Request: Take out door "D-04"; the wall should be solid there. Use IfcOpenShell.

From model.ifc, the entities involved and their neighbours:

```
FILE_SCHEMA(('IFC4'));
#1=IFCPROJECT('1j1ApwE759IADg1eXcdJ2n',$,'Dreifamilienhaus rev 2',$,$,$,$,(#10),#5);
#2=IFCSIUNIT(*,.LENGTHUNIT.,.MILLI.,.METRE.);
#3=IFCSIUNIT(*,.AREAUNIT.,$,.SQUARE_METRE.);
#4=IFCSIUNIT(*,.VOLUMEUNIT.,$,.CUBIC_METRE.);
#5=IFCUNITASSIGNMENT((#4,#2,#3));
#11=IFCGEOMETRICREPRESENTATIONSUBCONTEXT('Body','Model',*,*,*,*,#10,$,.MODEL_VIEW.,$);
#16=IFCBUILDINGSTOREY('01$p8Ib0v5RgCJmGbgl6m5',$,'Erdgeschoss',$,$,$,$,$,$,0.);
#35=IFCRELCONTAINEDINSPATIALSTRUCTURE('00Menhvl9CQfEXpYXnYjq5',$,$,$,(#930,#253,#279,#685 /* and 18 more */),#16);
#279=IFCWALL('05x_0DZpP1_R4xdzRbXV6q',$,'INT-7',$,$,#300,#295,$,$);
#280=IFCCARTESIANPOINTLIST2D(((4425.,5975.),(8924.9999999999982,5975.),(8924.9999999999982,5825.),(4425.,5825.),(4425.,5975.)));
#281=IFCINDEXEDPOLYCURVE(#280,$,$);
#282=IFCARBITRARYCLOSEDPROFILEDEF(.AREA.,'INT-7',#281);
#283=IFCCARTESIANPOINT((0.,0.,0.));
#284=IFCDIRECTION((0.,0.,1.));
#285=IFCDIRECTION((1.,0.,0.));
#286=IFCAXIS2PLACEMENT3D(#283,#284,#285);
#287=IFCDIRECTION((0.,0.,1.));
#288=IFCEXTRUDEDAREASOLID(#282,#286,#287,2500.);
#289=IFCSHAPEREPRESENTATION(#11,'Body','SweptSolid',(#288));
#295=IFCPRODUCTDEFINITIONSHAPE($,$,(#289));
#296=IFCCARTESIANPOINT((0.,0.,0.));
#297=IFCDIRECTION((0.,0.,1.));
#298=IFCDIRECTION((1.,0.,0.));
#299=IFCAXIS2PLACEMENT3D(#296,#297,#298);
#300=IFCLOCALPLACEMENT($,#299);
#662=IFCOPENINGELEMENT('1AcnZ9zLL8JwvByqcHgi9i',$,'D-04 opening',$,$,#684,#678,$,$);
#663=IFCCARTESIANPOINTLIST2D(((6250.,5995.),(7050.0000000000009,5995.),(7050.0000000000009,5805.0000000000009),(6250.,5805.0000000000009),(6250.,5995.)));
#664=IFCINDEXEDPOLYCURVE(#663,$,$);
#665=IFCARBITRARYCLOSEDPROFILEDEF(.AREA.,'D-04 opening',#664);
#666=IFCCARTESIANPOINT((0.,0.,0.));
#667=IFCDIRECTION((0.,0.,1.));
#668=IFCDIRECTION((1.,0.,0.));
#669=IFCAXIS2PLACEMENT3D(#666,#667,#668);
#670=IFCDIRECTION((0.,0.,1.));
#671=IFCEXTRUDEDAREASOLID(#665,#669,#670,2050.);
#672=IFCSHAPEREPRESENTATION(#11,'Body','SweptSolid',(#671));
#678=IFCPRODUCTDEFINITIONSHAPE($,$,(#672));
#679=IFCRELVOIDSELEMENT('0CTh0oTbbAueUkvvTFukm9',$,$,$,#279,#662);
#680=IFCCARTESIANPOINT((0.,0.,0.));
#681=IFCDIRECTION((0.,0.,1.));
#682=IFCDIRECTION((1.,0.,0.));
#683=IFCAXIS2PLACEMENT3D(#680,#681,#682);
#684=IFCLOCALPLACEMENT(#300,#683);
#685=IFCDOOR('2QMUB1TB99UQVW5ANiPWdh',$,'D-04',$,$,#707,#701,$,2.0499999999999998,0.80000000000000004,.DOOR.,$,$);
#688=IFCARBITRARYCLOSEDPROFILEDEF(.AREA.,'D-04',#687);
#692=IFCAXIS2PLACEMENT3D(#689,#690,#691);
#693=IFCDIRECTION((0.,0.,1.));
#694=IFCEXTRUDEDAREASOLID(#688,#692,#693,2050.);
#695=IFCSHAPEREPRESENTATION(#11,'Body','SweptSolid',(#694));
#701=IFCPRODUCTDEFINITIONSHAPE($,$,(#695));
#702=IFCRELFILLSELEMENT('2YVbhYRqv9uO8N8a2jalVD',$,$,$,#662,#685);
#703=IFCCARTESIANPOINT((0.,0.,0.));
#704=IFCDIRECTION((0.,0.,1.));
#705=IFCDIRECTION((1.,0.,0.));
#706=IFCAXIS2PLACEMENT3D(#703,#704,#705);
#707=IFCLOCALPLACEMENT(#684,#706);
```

```python
import ifcopenshell
import ifcopenshell.api.feature
import ifcopenshell.api.root
import ifcopenshell.geom
import ifcopenshell.util.shape

model = ifcopenshell.open("model.ifc")
settings = ifcopenshell.geom.settings()


def volume(element):
    """Net volume in cubic metres, openings subtracted."""
    shape = ifcopenshell.geom.create_shape(settings, element)
    return ifcopenshell.util.shape.get_volume(shape.geometry)


door = model.by_guid("2QMUB1TB99UQVW5ANiPWdh")
opening = door.FillsVoids[0].RelatingOpeningElement
wall = opening.VoidsElements[0].RelatingBuildingElement
before = volume(wall)

ifcopenshell.api.root.remove_product(model, product=door)
ifcopenshell.api.feature.remove_feature(model, feature=opening)

after = volume(wall)

print(f"wall volume {before:.3f} -> {after:.3f} m3")

model.write("model_v2.ifc")
```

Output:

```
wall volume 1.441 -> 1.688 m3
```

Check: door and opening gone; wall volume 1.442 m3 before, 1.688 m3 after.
